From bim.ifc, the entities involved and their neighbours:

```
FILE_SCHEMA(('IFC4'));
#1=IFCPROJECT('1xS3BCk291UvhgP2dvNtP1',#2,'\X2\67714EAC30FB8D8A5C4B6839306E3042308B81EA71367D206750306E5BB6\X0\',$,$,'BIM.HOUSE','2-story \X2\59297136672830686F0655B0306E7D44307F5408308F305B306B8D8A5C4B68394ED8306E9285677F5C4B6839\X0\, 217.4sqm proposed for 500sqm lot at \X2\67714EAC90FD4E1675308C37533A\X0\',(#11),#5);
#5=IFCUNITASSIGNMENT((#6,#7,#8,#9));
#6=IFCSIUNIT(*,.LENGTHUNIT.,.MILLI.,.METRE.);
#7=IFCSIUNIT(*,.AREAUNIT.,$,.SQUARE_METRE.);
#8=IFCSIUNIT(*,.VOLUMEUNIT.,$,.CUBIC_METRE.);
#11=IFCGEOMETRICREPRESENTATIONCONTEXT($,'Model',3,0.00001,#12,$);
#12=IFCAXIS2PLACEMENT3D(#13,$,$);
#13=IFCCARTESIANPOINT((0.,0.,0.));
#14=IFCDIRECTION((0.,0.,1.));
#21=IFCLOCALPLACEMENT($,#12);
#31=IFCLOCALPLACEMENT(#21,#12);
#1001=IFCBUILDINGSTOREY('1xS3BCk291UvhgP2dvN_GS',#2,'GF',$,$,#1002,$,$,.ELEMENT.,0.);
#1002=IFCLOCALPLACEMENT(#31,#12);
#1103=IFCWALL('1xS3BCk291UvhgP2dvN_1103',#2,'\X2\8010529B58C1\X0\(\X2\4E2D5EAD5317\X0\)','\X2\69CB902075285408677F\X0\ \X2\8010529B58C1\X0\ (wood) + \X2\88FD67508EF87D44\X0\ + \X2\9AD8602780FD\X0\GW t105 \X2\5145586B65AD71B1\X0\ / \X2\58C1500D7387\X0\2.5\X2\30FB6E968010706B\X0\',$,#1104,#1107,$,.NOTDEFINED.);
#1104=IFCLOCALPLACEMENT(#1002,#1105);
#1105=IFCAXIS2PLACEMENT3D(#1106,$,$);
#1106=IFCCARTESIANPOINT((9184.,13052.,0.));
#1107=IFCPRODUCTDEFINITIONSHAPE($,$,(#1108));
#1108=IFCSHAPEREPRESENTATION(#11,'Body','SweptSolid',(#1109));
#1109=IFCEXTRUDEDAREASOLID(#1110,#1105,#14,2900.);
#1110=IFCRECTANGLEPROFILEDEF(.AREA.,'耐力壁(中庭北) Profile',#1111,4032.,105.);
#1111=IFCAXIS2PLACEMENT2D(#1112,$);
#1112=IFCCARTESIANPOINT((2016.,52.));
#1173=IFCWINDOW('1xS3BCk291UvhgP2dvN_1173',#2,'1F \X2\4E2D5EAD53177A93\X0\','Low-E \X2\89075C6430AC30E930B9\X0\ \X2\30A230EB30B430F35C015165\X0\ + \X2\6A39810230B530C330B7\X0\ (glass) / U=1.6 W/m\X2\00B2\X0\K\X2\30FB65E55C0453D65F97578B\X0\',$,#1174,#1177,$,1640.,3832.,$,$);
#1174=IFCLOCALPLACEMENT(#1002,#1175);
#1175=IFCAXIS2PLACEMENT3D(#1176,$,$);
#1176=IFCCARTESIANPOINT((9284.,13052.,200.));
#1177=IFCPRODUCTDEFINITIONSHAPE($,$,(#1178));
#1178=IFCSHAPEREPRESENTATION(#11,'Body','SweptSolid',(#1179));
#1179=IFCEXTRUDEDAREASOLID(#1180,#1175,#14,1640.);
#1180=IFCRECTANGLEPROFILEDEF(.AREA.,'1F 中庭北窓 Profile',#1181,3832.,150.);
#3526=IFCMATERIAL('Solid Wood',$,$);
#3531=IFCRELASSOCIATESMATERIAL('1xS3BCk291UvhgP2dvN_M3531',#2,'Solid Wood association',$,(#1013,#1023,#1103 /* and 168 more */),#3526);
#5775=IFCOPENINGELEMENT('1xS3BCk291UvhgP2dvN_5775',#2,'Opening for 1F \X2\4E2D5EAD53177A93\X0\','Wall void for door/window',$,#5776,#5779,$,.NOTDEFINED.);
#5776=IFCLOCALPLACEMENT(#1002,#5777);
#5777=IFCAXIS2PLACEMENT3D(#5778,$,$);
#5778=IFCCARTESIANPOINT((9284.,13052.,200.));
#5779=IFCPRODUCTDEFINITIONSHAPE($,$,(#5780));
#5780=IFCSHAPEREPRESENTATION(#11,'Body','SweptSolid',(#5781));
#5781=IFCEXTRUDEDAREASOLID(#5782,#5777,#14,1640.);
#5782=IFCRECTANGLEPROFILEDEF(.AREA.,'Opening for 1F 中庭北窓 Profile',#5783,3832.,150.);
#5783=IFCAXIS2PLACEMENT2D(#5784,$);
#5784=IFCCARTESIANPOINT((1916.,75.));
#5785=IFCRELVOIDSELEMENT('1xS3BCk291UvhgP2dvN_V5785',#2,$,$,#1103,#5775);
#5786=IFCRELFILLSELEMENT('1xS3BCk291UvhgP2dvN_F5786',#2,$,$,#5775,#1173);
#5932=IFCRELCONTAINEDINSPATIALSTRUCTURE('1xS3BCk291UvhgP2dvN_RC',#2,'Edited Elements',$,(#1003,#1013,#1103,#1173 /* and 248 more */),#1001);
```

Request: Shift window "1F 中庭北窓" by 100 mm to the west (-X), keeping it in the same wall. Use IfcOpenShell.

```python
import ifcopenshell
import ifcopenshell.api.geometry
import ifcopenshell.util.placement
import ifcopenshell.util.unit

model = ifcopenshell.open("bim.ifc")
unit_scale = ifcopenshell.util.unit.calculate_unit_scale(model)

window = model.by_id(1173)
opening = window.FillsVoids[0].RelatingOpeningElement
wall = opening.VoidsElements[0].RelatingBuildingElement

wall_matrix = ifcopenshell.util.placement.get_local_placement(wall.ObjectPlacement)
shift = wall_matrix[:3, 0] * -0.1 / unit_scale
before = ifcopenshell.util.placement.get_local_placement(window.ObjectPlacement)[:3, 3].copy()

# The window is not placed relative to its opening, so move both.
for product in (opening, window):
    matrix = ifcopenshell.util.placement.get_local_placement(product.ObjectPlacement)
    matrix[:3, 3] += shift
    ifcopenshell.api.geometry.edit_object_placement(model, product=product, matrix=matrix, is_si=False)

after = ifcopenshell.util.placement.get_local_placement(window.ObjectPlacement)[:3, 3]
print("window moved by", (after - before).round(3) + 0.0)

model.write("bim-out.ifc")
```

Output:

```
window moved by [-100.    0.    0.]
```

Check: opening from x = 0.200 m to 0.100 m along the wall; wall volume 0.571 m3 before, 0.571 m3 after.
